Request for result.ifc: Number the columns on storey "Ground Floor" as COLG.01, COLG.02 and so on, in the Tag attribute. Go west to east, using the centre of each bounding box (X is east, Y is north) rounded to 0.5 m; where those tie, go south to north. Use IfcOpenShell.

First a look at what the model holds.

```python
import ifcopenshell
import ifcopenshell.util.element
import ifcopenshell.util.placement

model = ifcopenshell.open("result.ifc")
print(model.schema)
storey = next(s for s in model.by_type("IfcBuildingStorey") if s.Name == "Ground Floor")
columns = [e for e in ifcopenshell.util.element.get_decomposition(storey) if e.is_a("IfcColumn")]
for e in sorted(columns, key=lambda e: e.id()):
    origin = ifcopenshell.util.placement.get_local_placement(e.ObjectPlacement)[:3, 3]
    print(e.id(), e.Tag, e.Name, origin.round(2) + 0.0, sep=" | ")
```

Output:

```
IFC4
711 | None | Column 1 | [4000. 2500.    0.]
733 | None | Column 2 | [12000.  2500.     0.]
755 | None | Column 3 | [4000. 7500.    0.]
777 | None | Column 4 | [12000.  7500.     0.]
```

```python
import ifcopenshell
import ifcopenshell.geom
import ifcopenshell.util.element
import ifcopenshell.util.shape

model = ifcopenshell.open("result.ifc")
settings = ifcopenshell.geom.settings()
settings.set("use-world-coords", True)


def centre(element):
    shape = ifcopenshell.geom.create_shape(settings, element)
    return ifcopenshell.util.shape.get_bbox_centroid(shape.geometry)


storey = next(s for s in model.by_type("IfcBuildingStorey") if s.Name == "Ground Floor")
columns = [e for e in ifcopenshell.util.element.get_decomposition(storey) if e.is_a("IfcColumn")]

# Insertion points can sit at a corner or the storey origin, so sort by the geometry (in metres).
centres = {e: centre(e) for e in columns}
columns.sort(key=lambda e: (round(centres[e][0] / 0.5), centres[e][1]))

for i, e in enumerate(columns, start=1):
    number = f"COLG.{i:02d}"
    e.Tag = number
    print(e.id(), number)

model.write("result_rev.ifc")
```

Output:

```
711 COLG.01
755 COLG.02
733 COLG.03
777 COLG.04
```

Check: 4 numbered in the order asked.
